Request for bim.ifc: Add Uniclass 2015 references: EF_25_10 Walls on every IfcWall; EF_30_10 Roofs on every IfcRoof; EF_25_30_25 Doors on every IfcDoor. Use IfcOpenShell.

First a look at what the model holds.

```python
import ifcopenshell

model = ifcopenshell.open("bim.ifc")
print(model.schema)
print("classifications:", [c.Name for c in model.by_type("IfcClassification")])
for ifc_class in ("IfcDoor", "IfcRoof", "IfcStair", "IfcWall", "IfcWindow"):
    print(ifc_class, len(model.by_type(ifc_class)))
```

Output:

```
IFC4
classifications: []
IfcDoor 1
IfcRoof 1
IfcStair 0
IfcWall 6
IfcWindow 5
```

```python
import ifcopenshell
import ifcopenshell.api.classification

model = ifcopenshell.open("bim.ifc")

system = ifcopenshell.api.classification.add_classification(model, classification="Uniclass 2015")

codes = {
    "IfcWall": ("EF_25_10", "Walls"),
    "IfcRoof": ("EF_30_10", "Roofs"),
    "IfcDoor": ("EF_25_30_25", "Doors"),
}
for ifc_class, (code, name) in codes.items():
    products = model.by_type(ifc_class)
    ifcopenshell.api.classification.add_reference(
        model, products=products, classification=system, identification=code, name=name
    )
    print(code, len(products))

model.write("bim-out.ifc")
```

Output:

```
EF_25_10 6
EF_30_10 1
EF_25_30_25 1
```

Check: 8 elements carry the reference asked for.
